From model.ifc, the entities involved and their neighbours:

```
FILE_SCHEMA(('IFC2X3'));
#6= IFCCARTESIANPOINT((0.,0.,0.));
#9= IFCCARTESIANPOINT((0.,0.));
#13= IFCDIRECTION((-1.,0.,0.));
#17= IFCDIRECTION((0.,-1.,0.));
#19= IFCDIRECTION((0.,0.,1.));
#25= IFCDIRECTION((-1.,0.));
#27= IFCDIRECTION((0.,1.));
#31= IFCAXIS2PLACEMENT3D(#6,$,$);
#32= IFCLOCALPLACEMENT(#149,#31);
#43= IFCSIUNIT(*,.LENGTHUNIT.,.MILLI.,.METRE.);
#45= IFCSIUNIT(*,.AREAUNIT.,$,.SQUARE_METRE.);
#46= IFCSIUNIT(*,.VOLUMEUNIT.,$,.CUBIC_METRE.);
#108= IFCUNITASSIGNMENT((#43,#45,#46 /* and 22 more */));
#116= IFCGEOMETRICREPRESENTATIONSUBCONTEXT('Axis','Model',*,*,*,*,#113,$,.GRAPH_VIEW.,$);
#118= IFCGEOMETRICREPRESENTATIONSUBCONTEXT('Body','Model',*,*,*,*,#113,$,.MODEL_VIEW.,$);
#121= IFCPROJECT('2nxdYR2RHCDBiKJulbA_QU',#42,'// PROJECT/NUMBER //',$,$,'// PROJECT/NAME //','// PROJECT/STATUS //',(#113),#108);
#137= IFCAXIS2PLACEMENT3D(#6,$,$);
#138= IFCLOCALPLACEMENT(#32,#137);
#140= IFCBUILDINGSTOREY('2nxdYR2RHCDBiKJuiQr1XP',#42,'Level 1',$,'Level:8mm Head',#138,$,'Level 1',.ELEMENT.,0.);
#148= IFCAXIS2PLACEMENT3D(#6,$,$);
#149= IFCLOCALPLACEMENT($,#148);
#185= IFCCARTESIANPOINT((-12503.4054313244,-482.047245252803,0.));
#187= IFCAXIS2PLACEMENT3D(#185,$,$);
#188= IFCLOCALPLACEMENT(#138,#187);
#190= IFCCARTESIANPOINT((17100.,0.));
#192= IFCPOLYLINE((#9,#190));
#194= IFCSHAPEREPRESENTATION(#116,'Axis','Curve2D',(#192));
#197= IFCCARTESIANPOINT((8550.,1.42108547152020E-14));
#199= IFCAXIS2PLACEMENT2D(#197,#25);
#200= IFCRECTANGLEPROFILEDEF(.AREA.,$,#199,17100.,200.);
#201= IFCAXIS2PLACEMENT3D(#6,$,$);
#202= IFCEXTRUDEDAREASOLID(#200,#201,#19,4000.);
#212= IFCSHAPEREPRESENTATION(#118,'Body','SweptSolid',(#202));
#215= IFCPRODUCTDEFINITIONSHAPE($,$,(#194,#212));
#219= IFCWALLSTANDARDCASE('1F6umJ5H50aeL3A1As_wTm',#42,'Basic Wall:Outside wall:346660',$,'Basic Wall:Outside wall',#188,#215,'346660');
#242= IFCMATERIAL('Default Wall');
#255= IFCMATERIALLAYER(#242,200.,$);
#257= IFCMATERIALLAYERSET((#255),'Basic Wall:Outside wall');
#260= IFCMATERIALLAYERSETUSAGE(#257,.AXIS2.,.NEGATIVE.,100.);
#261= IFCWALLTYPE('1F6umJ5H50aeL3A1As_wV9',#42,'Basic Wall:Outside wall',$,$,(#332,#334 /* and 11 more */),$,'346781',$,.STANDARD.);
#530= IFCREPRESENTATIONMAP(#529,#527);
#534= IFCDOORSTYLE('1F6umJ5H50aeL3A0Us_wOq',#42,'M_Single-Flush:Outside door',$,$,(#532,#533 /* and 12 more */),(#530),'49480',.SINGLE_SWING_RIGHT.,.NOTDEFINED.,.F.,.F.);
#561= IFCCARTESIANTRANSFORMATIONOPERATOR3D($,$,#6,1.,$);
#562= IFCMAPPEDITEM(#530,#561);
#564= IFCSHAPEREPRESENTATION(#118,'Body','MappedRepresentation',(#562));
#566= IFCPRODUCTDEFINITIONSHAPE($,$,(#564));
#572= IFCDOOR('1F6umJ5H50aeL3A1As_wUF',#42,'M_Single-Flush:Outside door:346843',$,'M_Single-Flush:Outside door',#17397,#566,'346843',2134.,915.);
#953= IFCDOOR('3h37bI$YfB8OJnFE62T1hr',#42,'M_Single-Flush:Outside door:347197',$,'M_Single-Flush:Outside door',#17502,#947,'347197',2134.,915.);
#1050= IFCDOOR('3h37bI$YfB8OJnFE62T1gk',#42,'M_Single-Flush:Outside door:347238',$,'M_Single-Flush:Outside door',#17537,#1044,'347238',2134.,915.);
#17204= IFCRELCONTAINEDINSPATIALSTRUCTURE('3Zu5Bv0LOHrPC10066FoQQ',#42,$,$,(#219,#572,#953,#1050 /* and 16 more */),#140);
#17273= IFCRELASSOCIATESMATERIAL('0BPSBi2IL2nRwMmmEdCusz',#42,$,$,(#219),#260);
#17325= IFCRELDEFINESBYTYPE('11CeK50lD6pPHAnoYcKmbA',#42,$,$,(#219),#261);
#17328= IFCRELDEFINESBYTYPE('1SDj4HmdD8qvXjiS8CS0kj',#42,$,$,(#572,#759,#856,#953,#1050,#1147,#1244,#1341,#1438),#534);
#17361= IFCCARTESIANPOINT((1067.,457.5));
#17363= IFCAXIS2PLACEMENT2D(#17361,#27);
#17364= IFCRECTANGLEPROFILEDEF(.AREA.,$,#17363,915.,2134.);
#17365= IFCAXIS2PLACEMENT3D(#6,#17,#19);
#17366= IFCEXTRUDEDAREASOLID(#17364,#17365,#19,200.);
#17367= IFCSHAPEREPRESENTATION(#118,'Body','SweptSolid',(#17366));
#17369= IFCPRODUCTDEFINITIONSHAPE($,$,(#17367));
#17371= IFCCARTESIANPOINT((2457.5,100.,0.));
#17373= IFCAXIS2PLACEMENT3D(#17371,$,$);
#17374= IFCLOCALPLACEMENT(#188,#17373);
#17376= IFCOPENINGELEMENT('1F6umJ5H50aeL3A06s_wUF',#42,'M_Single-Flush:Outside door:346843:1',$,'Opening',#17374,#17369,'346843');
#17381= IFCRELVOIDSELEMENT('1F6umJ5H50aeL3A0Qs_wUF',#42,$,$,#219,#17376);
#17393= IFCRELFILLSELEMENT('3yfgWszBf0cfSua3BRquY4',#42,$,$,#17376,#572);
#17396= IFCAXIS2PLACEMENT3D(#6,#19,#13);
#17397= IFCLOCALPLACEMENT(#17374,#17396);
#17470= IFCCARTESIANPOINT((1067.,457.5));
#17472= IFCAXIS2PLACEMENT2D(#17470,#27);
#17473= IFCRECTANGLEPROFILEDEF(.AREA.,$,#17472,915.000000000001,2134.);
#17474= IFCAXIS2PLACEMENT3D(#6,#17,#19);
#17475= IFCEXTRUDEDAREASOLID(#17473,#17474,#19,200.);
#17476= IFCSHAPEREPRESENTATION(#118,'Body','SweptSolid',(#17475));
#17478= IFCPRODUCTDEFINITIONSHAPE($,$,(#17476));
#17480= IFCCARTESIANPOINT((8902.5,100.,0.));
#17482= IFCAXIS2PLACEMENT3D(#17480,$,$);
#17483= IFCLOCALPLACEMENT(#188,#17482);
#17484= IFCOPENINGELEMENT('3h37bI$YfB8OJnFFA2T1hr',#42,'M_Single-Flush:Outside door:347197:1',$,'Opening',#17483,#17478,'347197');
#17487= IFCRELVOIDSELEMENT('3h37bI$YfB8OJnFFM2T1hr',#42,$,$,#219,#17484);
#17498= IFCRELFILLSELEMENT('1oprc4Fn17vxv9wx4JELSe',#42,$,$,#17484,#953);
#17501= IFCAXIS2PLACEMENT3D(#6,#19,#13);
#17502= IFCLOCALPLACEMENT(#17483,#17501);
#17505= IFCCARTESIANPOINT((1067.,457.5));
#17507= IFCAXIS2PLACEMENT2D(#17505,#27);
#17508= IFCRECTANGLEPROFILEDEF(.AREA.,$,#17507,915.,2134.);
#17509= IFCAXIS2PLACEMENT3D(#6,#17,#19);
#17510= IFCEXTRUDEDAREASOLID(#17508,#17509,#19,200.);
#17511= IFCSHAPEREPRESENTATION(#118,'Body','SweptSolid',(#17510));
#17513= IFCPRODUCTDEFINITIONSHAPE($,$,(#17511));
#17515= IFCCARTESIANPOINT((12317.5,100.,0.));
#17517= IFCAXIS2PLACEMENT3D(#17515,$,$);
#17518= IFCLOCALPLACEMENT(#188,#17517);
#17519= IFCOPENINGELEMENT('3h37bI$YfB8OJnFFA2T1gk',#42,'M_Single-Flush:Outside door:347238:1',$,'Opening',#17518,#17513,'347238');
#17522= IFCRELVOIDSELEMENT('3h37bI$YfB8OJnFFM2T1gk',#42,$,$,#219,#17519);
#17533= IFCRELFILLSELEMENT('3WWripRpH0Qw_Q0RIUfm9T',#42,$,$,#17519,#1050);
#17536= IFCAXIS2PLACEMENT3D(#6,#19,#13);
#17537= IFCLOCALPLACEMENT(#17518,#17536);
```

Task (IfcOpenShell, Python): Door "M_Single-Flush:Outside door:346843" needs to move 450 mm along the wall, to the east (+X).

```python
import ifcopenshell
import ifcopenshell.api.geometry
import ifcopenshell.util.placement

model = ifcopenshell.open("model.ifc")

door = model.by_guid("1F6umJ5H50aeL3A1As_wUF")
opening = door.FillsVoids[0].RelatingOpeningElement
wall = opening.VoidsElements[0].RelatingBuildingElement

wall_matrix = ifcopenshell.util.placement.get_local_placement(wall.ObjectPlacement)
shift = wall_matrix[:3, 0] * 450.0
before = ifcopenshell.util.placement.get_local_placement(door.ObjectPlacement)[:3, 3].copy()

# The door is placed relative to its opening, so it follows when the opening moves.
matrix = ifcopenshell.util.placement.get_local_placement(opening.ObjectPlacement)
matrix[:3, 3] += shift
ifcopenshell.api.geometry.edit_object_placement(
    model, product=opening, matrix=matrix, is_si=False, should_transform_children=True
)

after = ifcopenshell.util.placement.get_local_placement(door.ObjectPlacement)[:3, 3]
print("door moved by", (after - before).round(3) + 0.0)

model.write("model_updated.ifc")
```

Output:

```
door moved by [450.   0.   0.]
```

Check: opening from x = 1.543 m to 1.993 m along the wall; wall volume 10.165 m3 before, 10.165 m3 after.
